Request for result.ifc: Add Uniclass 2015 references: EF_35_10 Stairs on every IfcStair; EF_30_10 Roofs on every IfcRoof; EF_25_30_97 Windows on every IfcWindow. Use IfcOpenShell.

First a look at what the model holds.

```python
import ifcopenshell

model = ifcopenshell.open("result.ifc")
print(model.schema)
print("classifications:", [c.Name for c in model.by_type("IfcClassification")])
for ifc_class in ("IfcDoor", "IfcRoof", "IfcStair", "IfcWall", "IfcWindow"):
    print(ifc_class, len(model.by_type(ifc_class)))
```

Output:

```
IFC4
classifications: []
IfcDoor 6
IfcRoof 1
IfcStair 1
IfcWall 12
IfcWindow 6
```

```python
import ifcopenshell
import ifcopenshell.api.classification

model = ifcopenshell.open("result.ifc")

system = ifcopenshell.api.classification.add_classification(model, classification="Uniclass 2015")

codes = {
    "IfcStair": ("EF_35_10", "Stairs"),
    "IfcRoof": ("EF_30_10", "Roofs"),
    "IfcWindow": ("EF_25_30_97", "Windows"),
}
for ifc_class, (code, name) in codes.items():
    products = model.by_type(ifc_class)
    ifcopenshell.api.classification.add_reference(
        model, products=products, classification=system, identification=code, name=name
    )
    print(code, len(products))

model.write("result-out.ifc")
```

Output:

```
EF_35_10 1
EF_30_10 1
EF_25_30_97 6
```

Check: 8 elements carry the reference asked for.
